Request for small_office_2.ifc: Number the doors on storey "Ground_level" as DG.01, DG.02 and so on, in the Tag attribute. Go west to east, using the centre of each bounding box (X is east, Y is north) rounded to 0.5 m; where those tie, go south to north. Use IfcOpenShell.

First a look at what the model holds.

```python
import ifcopenshell
import ifcopenshell.util.element
import ifcopenshell.util.placement

model = ifcopenshell.open("small_office_2.ifc")
print(model.schema)
storey = next(s for s in model.by_type("IfcBuildingStorey") if s.Name == "Ground_level")
doors = [e for e in ifcopenshell.util.element.get_decomposition(storey) if e.is_a("IfcDoor")]
for e in sorted(doors, key=lambda e: e.id()):
    origin = ifcopenshell.util.placement.get_local_placement(e.ObjectPlacement)[:3, 3]
    print(e.id(), e.Tag, e.Name, origin.round(2) + 0.0, sep=" | ")
```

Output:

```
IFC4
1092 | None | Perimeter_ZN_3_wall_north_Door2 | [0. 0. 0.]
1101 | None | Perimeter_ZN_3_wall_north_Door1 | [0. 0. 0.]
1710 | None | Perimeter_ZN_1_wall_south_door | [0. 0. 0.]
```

```python
import ifcopenshell
import ifcopenshell.geom
import ifcopenshell.util.element
import ifcopenshell.util.shape

model = ifcopenshell.open("small_office_2.ifc")
settings = ifcopenshell.geom.settings()
settings.set("use-world-coords", True)


def centre(element):
    shape = ifcopenshell.geom.create_shape(settings, element)
    return ifcopenshell.util.shape.get_bbox_centroid(shape.geometry)


storey = next(s for s in model.by_type("IfcBuildingStorey") if s.Name == "Ground_level")
doors = [e for e in ifcopenshell.util.element.get_decomposition(storey) if e.is_a("IfcDoor")]

# Insertion points can sit at a corner or the storey origin, so sort by the geometry (in metres).
centres = {e: centre(e) for e in doors}
doors.sort(key=lambda e: (round(centres[e][0] / 0.5), centres[e][1]))

for i, e in enumerate(doors, start=1):
    number = f"DG.{i:02d}"
    e.Tag = number
    print(e.id(), number)

model.write("small_office_2_rev.ifc")
```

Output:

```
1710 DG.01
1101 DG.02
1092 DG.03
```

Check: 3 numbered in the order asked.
